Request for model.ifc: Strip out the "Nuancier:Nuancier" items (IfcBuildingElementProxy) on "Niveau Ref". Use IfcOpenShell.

First a look at what the model holds.

```python
import ifcopenshell
import ifcopenshell.util.element

model = ifcopenshell.open("model.ifc")
print(model.schema)
storey = next(s for s in model.by_type("IfcBuildingStorey") if s.Name == "Niveau Ref")
proxies = [e for e in ifcopenshell.util.element.get_decomposition(storey) if e.is_a("IfcBuildingElementProxy")]
seen = {}
for e in proxies:
    element_type = ifcopenshell.util.element.get_type(e)
    name = element_type.Name if element_type not in (None, e) else None
    seen[name] = seen.get(name, 0) + 1
for name, count in sorted(seen.items(), key=str):
    print(count, "x", name)
```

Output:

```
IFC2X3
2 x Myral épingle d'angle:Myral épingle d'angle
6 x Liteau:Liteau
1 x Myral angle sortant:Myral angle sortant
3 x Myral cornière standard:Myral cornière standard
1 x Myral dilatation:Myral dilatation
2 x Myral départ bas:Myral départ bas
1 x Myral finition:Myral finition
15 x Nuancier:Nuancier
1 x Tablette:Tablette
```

```python
import ifcopenshell
import ifcopenshell.api.root
import ifcopenshell.util.element

model = ifcopenshell.open("model.ifc")

storey = next(s for s in model.by_type("IfcBuildingStorey") if s.Name == "Niveau Ref")
proxies = [e for e in ifcopenshell.util.element.get_decomposition(storey) if e.is_a("IfcBuildingElementProxy")]
targets = [e for e in proxies if (t := ifcopenshell.util.element.get_type(e)) not in (None, e) and t.Name == "Nuancier:Nuancier"]

for e in targets:
    ifcopenshell.api.root.remove_product(model, product=e)
print(len(targets), "removed")

model.write("model_rev.ifc")
```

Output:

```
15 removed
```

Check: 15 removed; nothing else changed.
